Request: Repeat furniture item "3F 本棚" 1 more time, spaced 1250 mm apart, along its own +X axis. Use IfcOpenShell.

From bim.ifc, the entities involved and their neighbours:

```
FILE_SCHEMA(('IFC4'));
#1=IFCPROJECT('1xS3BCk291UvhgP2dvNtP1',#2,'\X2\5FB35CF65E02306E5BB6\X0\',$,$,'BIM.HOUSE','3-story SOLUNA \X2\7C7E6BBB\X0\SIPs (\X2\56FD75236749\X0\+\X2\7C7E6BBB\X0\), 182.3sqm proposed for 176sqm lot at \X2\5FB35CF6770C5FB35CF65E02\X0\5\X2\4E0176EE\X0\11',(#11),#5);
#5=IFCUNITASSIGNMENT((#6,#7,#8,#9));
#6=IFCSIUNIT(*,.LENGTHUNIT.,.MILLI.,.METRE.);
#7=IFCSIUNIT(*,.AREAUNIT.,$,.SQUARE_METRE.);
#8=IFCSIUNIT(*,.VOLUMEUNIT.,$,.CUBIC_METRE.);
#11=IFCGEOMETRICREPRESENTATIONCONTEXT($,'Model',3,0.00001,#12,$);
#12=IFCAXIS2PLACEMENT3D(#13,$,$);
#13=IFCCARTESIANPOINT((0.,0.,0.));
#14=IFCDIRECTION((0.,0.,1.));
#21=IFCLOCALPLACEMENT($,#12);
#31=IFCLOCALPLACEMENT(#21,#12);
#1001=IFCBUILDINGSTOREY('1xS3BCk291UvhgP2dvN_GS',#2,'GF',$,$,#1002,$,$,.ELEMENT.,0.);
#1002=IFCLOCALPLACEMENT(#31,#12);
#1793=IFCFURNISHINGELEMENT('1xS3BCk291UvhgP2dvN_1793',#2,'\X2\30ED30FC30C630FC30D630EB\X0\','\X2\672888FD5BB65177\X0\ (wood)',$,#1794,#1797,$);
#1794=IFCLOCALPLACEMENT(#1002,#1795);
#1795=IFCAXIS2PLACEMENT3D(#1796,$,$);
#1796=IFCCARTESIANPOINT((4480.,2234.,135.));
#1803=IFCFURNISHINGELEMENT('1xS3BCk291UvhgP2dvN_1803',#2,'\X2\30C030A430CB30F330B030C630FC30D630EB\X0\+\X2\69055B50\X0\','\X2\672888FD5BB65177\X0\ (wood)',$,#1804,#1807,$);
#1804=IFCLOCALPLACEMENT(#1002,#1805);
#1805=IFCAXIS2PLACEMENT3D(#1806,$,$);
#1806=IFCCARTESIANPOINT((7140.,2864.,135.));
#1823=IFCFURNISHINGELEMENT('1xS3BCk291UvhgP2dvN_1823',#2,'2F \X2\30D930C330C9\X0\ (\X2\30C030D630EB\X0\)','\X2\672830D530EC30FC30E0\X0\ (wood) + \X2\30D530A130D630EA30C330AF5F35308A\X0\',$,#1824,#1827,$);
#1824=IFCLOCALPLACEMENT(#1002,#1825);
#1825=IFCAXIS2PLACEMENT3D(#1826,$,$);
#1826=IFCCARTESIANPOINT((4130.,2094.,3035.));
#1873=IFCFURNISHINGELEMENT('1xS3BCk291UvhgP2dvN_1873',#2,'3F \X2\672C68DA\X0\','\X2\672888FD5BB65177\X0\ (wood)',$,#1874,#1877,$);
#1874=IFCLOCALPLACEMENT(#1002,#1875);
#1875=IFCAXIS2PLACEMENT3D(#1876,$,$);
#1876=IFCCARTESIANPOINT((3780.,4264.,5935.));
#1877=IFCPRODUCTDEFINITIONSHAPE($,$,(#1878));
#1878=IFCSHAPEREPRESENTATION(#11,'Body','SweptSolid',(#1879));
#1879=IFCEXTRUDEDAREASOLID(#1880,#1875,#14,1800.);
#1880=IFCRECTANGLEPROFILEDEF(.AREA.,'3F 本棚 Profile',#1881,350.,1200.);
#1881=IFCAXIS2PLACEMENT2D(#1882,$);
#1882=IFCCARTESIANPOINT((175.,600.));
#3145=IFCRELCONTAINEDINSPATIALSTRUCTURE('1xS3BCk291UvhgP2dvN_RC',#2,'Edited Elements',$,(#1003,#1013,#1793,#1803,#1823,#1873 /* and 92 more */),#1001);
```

```python
import ifcopenshell
import ifcopenshell.api.geometry
import ifcopenshell.api.root
import ifcopenshell.util.element
import ifcopenshell.util.placement

model = ifcopenshell.open("bim.ifc")


def reuse_history(source, copy):
    """copy_class also copies each property set's owner history, people and application; keep the originals."""
    for rel in copy.IsDefinedBy:
        if rel.is_a("IfcRelDefinesByProperties") and (history := rel.RelatingPropertyDefinition.OwnerHistory):
            rel.RelatingPropertyDefinition.OwnerHistory = source.OwnerHistory
            ifcopenshell.util.element.remove_deep2(model, history)


source = model.by_id(1873)
base = ifcopenshell.util.placement.get_local_placement(source.ObjectPlacement)
step = base[:3, 0] * 1250.0

for i in range(1, 2):
    copy = ifcopenshell.api.root.copy_class(model, product=source)
    copy.Representation = ifcopenshell.util.element.copy_deep(
        model, source.Representation, exclude=["IfcGeometricRepresentationContext", "IfcRepresentationMap"]
    )
    reuse_history(source, copy)
    matrix = base.copy()
    matrix[:3, 3] += i * step
    print("added at", matrix[:3, 3].round(3) + 0.0)
    ifcopenshell.api.geometry.edit_object_placement(model, product=copy, matrix=matrix, is_si=False)

model.write("bim_updated.ifc")
```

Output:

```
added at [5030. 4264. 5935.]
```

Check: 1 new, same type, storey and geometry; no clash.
